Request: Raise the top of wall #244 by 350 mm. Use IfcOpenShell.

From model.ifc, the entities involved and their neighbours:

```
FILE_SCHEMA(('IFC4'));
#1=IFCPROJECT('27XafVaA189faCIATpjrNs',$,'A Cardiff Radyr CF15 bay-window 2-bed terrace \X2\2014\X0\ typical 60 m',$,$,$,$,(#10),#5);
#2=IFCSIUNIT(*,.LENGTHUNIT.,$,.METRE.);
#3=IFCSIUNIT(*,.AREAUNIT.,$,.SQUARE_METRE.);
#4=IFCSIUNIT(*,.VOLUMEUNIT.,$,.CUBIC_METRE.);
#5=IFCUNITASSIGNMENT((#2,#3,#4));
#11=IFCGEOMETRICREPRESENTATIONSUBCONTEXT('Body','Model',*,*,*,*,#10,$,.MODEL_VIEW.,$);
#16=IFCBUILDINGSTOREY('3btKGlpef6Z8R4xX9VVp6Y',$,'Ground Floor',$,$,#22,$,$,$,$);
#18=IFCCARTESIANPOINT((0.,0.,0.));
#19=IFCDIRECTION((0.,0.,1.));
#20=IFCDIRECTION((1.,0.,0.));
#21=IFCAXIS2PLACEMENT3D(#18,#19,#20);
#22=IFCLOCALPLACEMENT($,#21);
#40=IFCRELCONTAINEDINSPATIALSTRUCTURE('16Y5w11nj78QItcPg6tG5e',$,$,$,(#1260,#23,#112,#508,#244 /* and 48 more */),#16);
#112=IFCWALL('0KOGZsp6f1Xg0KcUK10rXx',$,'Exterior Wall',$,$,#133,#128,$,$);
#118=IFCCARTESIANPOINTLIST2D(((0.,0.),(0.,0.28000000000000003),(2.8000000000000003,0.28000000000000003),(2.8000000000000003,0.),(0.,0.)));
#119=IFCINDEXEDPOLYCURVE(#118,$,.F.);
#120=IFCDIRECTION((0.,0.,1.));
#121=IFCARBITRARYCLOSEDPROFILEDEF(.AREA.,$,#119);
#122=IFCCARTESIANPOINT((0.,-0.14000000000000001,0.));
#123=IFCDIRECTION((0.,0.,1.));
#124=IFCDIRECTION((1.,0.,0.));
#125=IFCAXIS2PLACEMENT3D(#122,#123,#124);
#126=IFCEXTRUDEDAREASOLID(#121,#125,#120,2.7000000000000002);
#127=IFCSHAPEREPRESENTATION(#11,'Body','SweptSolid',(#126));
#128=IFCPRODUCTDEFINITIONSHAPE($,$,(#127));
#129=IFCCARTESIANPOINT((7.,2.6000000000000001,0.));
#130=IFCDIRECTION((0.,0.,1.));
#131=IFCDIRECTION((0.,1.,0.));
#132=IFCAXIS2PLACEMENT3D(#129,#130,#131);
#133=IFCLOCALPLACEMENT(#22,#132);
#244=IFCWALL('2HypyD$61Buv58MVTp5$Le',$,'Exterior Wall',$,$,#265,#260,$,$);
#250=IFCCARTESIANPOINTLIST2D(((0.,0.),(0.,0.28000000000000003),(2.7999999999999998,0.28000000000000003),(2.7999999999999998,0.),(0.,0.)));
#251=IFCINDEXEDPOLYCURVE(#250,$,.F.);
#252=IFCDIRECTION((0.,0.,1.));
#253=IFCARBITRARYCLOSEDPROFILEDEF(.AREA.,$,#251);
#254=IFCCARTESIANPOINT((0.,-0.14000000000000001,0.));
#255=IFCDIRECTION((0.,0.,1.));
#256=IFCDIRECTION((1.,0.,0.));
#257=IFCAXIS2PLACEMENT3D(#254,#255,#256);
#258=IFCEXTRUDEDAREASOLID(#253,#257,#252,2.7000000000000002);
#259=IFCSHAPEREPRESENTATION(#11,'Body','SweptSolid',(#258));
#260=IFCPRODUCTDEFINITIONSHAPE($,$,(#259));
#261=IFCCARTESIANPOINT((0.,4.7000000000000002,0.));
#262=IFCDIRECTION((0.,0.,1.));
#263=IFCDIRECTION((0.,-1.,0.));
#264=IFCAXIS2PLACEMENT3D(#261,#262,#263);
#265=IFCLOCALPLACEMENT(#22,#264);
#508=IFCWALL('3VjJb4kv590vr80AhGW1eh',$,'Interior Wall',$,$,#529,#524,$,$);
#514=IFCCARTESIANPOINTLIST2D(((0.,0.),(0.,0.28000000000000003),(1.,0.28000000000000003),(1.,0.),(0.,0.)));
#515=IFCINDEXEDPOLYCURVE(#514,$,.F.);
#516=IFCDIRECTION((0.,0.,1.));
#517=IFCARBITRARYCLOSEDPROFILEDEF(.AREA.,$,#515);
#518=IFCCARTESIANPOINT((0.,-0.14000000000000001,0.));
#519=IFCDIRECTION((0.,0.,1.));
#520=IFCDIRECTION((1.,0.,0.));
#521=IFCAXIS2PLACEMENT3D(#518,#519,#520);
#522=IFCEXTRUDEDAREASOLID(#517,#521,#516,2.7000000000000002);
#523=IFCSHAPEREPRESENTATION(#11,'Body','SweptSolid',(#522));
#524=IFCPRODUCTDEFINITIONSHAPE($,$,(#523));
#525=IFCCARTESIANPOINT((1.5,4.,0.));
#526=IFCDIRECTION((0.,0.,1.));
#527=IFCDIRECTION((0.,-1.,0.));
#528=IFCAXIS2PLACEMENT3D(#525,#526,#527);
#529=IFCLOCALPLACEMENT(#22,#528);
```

```python
import ifcopenshell
import ifcopenshell.geom
import ifcopenshell.util.representation
import ifcopenshell.util.shape

model = ifcopenshell.open("model.ifc")
settings = ifcopenshell.geom.settings()


def volume(element):
    """Net volume in cubic metres, openings subtracted."""
    shape = ifcopenshell.geom.create_shape(settings, element)
    return ifcopenshell.util.shape.get_volume(shape.geometry)


wall = model.by_guid("2HypyD$61Buv58MVTp5$Le")
before = volume(wall)

body = ifcopenshell.util.representation.get_representation(wall, "Model", "Body")
solid = body.Items[0]
old_height = solid.Depth
solid.Depth += 0.35
after = volume(wall)

print(f"height {old_height:g} -> {solid.Depth:g}, volume {before:.3f} -> {after:.3f} m3")

model.write("model_edited.ifc")
```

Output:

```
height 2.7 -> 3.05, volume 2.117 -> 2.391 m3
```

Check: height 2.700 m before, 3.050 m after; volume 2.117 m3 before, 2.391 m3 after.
